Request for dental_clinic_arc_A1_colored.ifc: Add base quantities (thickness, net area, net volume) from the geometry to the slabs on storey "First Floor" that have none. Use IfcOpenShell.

First a look at what the model holds.

```python
import ifcopenshell
import ifcopenshell.util.element
import ifcopenshell.util.unit

model = ifcopenshell.open("dental_clinic_arc_A1_colored.ifc")
print(model.schema)
for unit_type in ("LENGTHUNIT", "AREAUNIT", "VOLUMEUNIT"):
    print(unit_type, ifcopenshell.util.unit.calculate_unit_scale(model, unit_type))
storey = next(s for s in model.by_type("IfcBuildingStorey") if s.Name == "First Floor")
slabs = [e for e in ifcopenshell.util.element.get_decomposition(storey) if e.is_a("IfcSlab")]
for e in sorted(slabs, key=lambda e: e.id()):
    print(e.id(), e.is_a(), e.Name, list(ifcopenshell.util.element.get_psets(e, qtos_only=True)), sep=" | ")
```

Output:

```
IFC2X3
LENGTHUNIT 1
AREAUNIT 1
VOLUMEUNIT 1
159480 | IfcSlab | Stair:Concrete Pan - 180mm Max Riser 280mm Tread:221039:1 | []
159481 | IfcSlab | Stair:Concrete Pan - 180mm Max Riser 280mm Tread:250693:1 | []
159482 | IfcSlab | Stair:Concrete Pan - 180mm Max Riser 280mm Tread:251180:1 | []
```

```python
import ifcopenshell
import ifcopenshell.api.pset
import ifcopenshell.geom
import ifcopenshell.util.element
import ifcopenshell.util.shape
import ifcopenshell.util.unit

model = ifcopenshell.open("dental_clinic_arc_A1_colored.ifc")
unit_scale = ifcopenshell.util.unit.calculate_unit_scale(model)
area_scale = ifcopenshell.util.unit.calculate_unit_scale(model, "AREAUNIT")
volume_scale = ifcopenshell.util.unit.calculate_unit_scale(model, "VOLUMEUNIT")
settings = ifcopenshell.geom.settings()

storey = next(s for s in model.by_type("IfcBuildingStorey") if s.Name == "First Floor")
slabs = [e for e in ifcopenshell.util.element.get_decomposition(storey) if e.is_a("IfcSlab")]

for e in sorted(slabs, key=lambda e: e.id()):
    if ifcopenshell.util.element.get_psets(e, qtos_only=True, should_inherit=False):
        continue
    # Geometry comes back in metres, in the element's own axes.
    shape = ifcopenshell.geom.create_shape(settings, e)
    values = {
        "Width": ifcopenshell.util.shape.get_z(shape.geometry) / unit_scale,
        "NetArea": ifcopenshell.util.shape.get_footprint_area(shape.geometry) / area_scale,
        "NetVolume": ifcopenshell.util.shape.get_volume(shape.geometry) / volume_scale,
    }
    qto = ifcopenshell.api.pset.add_qto(model, product=e, name="BaseQuantities")
    ifcopenshell.api.pset.edit_qto(model, qto=qto, properties=values)
    print(e.id(), {k: round(v, 3) for k, v in values.items()})

model.write("dental_clinic_arc_A1_colored_updated.ifc")
```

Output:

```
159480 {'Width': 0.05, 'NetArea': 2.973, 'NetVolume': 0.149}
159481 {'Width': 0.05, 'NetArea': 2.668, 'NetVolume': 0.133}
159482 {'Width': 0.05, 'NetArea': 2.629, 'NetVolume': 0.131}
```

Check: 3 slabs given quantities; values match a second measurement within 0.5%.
